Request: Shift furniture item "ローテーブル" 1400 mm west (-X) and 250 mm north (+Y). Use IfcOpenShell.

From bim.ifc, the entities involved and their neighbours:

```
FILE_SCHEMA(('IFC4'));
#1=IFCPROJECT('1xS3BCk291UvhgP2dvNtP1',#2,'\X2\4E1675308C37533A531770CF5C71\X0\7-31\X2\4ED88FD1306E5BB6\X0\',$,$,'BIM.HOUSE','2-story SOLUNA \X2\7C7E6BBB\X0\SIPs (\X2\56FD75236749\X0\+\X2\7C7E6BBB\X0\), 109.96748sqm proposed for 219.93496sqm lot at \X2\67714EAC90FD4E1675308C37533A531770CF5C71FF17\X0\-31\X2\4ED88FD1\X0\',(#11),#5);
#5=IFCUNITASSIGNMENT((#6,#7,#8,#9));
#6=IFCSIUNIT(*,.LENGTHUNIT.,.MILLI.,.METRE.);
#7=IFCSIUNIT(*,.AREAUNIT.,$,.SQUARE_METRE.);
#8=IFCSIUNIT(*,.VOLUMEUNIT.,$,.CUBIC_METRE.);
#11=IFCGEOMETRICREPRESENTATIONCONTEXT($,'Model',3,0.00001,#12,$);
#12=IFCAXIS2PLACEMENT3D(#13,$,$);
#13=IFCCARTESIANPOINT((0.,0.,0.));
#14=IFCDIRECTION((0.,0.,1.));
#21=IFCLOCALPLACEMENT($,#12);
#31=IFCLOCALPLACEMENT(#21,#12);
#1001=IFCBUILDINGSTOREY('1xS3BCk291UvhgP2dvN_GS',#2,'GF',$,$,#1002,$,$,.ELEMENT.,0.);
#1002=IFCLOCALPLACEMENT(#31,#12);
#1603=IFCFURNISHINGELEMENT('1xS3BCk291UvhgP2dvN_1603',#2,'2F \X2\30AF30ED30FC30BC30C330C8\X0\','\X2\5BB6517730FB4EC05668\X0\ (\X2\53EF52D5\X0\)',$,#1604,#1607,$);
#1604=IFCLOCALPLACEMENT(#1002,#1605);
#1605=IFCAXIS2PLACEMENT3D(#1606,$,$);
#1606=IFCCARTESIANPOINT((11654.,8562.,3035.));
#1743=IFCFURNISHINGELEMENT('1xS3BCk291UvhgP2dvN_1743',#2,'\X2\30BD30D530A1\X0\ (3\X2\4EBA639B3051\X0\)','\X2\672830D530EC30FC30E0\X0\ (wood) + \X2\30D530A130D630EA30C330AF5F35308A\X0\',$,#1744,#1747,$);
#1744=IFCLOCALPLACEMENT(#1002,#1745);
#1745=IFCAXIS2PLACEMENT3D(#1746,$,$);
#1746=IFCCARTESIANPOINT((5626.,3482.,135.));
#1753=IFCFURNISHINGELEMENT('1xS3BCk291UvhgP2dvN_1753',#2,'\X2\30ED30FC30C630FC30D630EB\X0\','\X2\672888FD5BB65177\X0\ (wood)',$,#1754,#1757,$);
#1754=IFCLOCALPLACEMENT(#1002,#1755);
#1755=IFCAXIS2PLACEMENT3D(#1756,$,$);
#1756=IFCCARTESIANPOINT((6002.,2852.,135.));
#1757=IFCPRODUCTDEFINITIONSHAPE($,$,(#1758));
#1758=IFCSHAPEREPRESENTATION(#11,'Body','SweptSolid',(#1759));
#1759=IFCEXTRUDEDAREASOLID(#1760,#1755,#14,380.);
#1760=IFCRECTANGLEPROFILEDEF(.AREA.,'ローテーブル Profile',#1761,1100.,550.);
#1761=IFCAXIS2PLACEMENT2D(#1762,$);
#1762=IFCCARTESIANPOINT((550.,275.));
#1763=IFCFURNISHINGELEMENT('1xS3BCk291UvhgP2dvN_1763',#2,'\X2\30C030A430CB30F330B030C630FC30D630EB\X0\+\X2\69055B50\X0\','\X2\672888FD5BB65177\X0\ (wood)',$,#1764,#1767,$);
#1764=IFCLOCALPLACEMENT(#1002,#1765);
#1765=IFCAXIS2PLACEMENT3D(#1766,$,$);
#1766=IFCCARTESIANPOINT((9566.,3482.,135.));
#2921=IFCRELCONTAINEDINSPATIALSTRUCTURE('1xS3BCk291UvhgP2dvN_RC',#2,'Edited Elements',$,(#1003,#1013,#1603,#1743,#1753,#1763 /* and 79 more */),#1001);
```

```python
import ifcopenshell
import ifcopenshell.api.geometry
import ifcopenshell.util.placement
import ifcopenshell.util.unit

model = ifcopenshell.open("bim.ifc")
unit_scale = ifcopenshell.util.unit.calculate_unit_scale(model)

item = model.by_guid("1xS3BCk291UvhgP2dvN_1753")
matrix = ifcopenshell.util.placement.get_local_placement(item.ObjectPlacement)
matrix[0, 3] -= 1.4 / unit_scale
matrix[1, 3] += 0.25 / unit_scale
ifcopenshell.api.geometry.edit_object_placement(model, product=item, matrix=matrix, is_si=False)

print(ifcopenshell.util.placement.get_local_placement(item.ObjectPlacement).round(3) + 0.0)

model.write("bim-out.ifc")
```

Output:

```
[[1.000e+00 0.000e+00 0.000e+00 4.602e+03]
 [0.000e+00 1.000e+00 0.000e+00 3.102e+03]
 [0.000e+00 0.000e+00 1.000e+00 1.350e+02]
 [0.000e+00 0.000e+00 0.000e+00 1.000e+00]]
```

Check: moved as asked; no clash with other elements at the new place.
